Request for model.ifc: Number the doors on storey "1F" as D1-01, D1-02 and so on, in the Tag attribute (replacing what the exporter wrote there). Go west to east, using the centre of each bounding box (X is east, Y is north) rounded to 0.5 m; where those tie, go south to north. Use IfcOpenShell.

First a look at what the model holds.

```python
import ifcopenshell
import ifcopenshell.util.element
import ifcopenshell.util.placement

model = ifcopenshell.open("model.ifc")
print(model.schema)
storey = next(s for s in model.by_type("IfcBuildingStorey") if s.Name == "1F")
doors = [e for e in ifcopenshell.util.element.get_decomposition(storey) if e.is_a("IfcDoor")]
for e in sorted(doors, key=lambda e: e.id()):
    origin = ifcopenshell.util.placement.get_local_placement(e.ObjectPlacement)[:3, 3]
    print(e.id(), e.Tag, e.Name, origin.round(2) + 0.0, sep=" | ")
```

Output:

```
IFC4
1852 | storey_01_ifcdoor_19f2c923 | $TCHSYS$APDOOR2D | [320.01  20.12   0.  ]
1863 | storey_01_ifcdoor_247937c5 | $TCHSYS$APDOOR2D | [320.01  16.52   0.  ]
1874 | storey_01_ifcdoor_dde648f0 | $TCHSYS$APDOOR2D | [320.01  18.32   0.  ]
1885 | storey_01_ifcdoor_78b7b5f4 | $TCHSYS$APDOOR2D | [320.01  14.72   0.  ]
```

```python
import ifcopenshell
import ifcopenshell.geom
import ifcopenshell.util.element
import ifcopenshell.util.shape

model = ifcopenshell.open("model.ifc")
settings = ifcopenshell.geom.settings()
settings.set("use-world-coords", True)


def centre(element):
    shape = ifcopenshell.geom.create_shape(settings, element)
    return ifcopenshell.util.shape.get_bbox_centroid(shape.geometry)


storey = next(s for s in model.by_type("IfcBuildingStorey") if s.Name == "1F")
doors = [e for e in ifcopenshell.util.element.get_decomposition(storey) if e.is_a("IfcDoor")]

# Insertion points can sit at a corner or the storey origin, so sort by the geometry (in metres).
centres = {e: centre(e) for e in doors}
doors.sort(key=lambda e: (round(centres[e][0] / 0.5), centres[e][1]))

for i, e in enumerate(doors, start=1):
    number = f"D1-{i:02d}"
    e.Tag = number
    print(e.id(), number)

model.write("model_rev.ifc")
```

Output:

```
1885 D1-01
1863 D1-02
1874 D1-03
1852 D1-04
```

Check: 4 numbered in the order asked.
